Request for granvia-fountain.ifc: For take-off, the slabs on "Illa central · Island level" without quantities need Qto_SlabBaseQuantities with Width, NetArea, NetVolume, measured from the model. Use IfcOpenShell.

First a look at what the model holds.

```python
import ifcopenshell
import ifcopenshell.util.element
import ifcopenshell.util.unit

model = ifcopenshell.open("granvia-fountain.ifc")
print(model.schema)
for unit_type in ("LENGTHUNIT", "AREAUNIT", "VOLUMEUNIT"):
    print(unit_type, ifcopenshell.util.unit.calculate_unit_scale(model, unit_type))
storey = next(s for s in model.by_type("IfcBuildingStorey") if s.Name == "Illa central · Island level")
slabs = [e for e in ifcopenshell.util.element.get_decomposition(storey) if e.is_a("IfcSlab")]
for e in sorted(slabs, key=lambda e: e.id()):
    print(e.id(), e.is_a(), e.Name, list(ifcopenshell.util.element.get_psets(e, qtos_only=True)), sep=" | ")
```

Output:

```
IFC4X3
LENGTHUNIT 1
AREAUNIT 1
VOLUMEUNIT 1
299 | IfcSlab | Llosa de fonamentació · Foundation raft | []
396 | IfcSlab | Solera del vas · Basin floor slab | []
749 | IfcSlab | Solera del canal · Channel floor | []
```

```python
import ifcopenshell
import ifcopenshell.api.pset
import ifcopenshell.geom
import ifcopenshell.util.element
import ifcopenshell.util.shape
import ifcopenshell.util.unit

model = ifcopenshell.open("granvia-fountain.ifc")
unit_scale = ifcopenshell.util.unit.calculate_unit_scale(model)
area_scale = ifcopenshell.util.unit.calculate_unit_scale(model, "AREAUNIT")
volume_scale = ifcopenshell.util.unit.calculate_unit_scale(model, "VOLUMEUNIT")
settings = ifcopenshell.geom.settings()

storey = next(s for s in model.by_type("IfcBuildingStorey") if s.Name == "Illa central · Island level")
slabs = [e for e in ifcopenshell.util.element.get_decomposition(storey) if e.is_a("IfcSlab")]

for e in sorted(slabs, key=lambda e: e.id()):
    if ifcopenshell.util.element.get_psets(e, qtos_only=True, should_inherit=False):
        continue
    # Geometry comes back in metres, in the element's own axes.
    shape = ifcopenshell.geom.create_shape(settings, e)
    values = {
        "Width": ifcopenshell.util.shape.get_z(shape.geometry) / unit_scale,
        "NetArea": ifcopenshell.util.shape.get_footprint_area(shape.geometry) / area_scale,
        "NetVolume": ifcopenshell.util.shape.get_volume(shape.geometry) / volume_scale,
    }
    qto = ifcopenshell.api.pset.add_qto(model, product=e, name="Qto_SlabBaseQuantities")
    ifcopenshell.api.pset.edit_qto(model, qto=qto, properties=values)
    print(e.id(), {k: round(v, 3) for k, v in values.items()})

model.write("granvia-fountain_edited.ifc")
```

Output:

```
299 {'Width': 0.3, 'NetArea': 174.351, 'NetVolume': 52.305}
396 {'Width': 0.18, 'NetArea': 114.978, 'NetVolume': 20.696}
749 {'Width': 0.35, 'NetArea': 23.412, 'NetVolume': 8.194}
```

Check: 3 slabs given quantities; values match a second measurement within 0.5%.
